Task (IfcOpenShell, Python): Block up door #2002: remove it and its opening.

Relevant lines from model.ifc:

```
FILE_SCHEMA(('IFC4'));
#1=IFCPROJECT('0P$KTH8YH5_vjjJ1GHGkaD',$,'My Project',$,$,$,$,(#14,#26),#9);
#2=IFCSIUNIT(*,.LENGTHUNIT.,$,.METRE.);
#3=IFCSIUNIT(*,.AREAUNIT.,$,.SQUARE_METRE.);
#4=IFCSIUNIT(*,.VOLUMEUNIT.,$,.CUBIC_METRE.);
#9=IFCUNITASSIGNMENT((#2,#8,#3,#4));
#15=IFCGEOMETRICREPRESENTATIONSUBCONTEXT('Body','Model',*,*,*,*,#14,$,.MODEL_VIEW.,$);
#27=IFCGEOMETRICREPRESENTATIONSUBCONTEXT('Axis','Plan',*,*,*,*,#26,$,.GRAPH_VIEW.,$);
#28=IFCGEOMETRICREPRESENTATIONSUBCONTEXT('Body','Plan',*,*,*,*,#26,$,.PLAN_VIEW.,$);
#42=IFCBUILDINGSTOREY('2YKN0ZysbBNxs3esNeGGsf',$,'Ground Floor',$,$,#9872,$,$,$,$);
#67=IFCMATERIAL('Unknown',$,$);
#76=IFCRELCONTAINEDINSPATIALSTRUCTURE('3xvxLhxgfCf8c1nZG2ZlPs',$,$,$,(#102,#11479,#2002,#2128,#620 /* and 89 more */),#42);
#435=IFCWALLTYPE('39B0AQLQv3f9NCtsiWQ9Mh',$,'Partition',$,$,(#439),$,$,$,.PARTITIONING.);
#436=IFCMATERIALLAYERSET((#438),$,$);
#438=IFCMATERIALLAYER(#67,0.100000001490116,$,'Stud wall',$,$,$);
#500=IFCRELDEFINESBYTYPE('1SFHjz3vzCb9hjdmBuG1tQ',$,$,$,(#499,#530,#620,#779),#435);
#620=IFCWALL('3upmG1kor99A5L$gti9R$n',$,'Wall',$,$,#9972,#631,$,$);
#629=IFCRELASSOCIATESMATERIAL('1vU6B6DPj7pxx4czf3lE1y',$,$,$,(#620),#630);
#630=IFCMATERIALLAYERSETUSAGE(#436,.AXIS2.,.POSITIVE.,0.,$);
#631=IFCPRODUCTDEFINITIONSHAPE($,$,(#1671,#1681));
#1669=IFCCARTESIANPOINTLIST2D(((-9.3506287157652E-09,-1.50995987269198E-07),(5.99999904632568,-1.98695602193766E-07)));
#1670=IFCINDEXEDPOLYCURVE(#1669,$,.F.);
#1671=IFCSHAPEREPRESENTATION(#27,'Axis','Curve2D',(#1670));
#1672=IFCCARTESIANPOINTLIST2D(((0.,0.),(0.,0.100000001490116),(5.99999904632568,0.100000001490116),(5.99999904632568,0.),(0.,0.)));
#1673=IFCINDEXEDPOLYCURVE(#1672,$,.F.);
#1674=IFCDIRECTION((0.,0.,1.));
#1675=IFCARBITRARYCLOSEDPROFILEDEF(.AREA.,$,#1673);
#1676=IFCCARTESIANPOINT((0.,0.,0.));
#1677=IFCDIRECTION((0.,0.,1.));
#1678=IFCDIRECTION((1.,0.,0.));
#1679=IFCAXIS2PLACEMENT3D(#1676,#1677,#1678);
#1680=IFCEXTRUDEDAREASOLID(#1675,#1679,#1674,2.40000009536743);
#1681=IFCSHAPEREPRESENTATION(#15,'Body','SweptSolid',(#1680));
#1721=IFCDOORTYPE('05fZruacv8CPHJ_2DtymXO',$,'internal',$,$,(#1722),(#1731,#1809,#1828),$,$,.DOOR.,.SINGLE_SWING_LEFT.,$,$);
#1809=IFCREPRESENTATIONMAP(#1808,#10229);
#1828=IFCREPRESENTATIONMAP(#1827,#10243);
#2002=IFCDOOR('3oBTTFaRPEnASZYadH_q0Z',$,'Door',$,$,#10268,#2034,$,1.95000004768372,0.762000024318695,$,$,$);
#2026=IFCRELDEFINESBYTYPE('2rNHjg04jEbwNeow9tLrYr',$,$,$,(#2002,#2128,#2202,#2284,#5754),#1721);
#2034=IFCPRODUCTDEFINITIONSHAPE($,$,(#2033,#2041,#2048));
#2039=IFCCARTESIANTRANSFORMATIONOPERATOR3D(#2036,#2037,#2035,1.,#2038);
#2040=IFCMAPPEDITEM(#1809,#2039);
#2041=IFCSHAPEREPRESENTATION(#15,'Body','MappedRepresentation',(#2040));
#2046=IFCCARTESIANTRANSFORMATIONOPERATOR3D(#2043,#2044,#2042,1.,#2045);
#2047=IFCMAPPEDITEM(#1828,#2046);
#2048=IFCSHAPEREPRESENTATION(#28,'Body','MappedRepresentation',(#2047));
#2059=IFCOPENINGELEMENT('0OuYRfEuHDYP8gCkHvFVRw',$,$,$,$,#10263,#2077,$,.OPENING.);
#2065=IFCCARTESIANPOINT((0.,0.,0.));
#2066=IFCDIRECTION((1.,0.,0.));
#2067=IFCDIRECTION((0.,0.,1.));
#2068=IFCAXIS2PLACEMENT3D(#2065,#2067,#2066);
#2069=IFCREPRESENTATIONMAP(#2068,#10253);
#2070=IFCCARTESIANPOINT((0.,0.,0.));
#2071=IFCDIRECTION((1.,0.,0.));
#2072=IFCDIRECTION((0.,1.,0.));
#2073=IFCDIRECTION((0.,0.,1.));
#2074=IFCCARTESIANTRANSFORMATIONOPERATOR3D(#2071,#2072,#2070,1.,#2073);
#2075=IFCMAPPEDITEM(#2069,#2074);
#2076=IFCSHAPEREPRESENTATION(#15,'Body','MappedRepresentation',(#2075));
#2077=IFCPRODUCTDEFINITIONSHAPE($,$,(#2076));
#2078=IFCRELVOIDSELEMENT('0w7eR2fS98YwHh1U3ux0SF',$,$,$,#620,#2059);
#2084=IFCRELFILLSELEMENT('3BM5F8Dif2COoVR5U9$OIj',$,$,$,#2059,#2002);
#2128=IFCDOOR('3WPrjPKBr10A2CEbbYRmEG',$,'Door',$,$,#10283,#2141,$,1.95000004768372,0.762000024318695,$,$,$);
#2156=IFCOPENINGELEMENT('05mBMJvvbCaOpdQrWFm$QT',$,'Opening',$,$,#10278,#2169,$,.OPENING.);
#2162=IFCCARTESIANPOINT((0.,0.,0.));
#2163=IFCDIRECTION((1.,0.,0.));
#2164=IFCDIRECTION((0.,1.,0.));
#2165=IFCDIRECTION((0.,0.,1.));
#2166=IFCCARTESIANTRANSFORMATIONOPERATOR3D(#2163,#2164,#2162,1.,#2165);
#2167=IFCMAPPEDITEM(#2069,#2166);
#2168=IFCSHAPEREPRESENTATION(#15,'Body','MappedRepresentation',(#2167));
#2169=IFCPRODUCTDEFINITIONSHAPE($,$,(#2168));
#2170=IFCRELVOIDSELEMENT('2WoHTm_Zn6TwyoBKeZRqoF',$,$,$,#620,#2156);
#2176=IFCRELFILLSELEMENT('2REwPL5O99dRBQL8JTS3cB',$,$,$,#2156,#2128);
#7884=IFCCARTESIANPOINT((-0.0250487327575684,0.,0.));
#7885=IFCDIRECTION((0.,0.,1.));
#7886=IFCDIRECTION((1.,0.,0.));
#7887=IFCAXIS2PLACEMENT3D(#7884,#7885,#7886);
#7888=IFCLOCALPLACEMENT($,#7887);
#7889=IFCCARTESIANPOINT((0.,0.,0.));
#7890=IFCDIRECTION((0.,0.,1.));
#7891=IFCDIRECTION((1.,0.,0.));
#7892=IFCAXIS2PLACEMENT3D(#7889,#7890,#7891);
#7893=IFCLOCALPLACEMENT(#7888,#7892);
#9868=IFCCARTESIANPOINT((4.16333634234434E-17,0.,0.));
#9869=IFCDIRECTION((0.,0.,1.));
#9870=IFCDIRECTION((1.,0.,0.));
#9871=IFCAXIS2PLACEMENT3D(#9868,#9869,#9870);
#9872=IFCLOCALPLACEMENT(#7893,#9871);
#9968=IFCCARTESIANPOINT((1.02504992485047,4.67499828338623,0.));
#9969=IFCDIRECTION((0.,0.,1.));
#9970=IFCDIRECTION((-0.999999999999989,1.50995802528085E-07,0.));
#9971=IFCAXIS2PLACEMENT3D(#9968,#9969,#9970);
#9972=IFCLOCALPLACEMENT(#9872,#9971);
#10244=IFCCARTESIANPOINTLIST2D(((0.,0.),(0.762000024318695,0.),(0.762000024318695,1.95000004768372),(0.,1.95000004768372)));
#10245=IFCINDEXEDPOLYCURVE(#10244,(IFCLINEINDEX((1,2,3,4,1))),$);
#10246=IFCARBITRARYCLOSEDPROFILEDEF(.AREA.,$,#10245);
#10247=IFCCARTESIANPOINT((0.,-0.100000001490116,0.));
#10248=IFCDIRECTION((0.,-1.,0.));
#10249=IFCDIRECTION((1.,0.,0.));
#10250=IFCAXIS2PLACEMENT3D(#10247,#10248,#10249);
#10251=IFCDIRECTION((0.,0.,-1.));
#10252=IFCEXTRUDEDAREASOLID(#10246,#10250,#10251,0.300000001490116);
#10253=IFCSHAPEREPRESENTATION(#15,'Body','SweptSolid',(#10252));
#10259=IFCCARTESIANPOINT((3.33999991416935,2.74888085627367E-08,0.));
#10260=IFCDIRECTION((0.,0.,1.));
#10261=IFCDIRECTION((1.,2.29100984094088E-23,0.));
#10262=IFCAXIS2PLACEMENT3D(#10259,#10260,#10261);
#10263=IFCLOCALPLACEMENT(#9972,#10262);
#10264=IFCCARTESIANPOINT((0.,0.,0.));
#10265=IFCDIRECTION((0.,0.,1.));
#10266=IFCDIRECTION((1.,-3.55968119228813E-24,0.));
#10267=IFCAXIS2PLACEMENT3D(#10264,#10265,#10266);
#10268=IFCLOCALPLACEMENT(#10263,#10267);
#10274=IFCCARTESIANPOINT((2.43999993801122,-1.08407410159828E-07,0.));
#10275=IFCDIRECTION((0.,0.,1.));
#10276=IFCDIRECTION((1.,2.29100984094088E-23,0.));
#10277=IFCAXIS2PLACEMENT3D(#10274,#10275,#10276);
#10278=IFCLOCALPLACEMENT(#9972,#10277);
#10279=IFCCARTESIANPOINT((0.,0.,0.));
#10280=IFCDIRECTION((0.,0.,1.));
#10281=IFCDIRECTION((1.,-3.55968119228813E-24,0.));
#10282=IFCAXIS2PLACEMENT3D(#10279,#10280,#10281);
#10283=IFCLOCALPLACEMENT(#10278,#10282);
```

```python
import ifcopenshell
import ifcopenshell.api.feature
import ifcopenshell.api.root
import ifcopenshell.geom
import ifcopenshell.util.shape

model = ifcopenshell.open("model.ifc")
settings = ifcopenshell.geom.settings()


def volume(element):
    """Net volume in cubic metres, openings subtracted."""
    shape = ifcopenshell.geom.create_shape(settings, element)
    return ifcopenshell.util.shape.get_volume(shape.geometry)


door = model.by_id(2002)
opening = door.FillsVoids[0].RelatingOpeningElement
wall = opening.VoidsElements[0].RelatingBuildingElement
before = volume(wall)

ifcopenshell.api.root.remove_product(model, product=door)
ifcopenshell.api.feature.remove_feature(model, feature=opening)

after = volume(wall)

print(f"wall volume {before:.3f} -> {after:.3f} m3")

model.write("model_edited.ifc")
```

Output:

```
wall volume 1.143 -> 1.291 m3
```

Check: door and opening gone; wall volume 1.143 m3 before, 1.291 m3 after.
